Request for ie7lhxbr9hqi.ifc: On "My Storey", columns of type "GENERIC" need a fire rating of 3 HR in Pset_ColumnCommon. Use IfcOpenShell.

First a look at what the model holds.

```python
import ifcopenshell
import ifcopenshell.util.element

model = ifcopenshell.open("ie7lhxbr9hqi.ifc")
print(model.schema)
storey = next(s for s in model.by_type("IfcBuildingStorey") if s.Name == "My Storey")
columns = [e for e in ifcopenshell.util.element.get_decomposition(storey) if e.is_a("IfcColumn")]
seen = {}
for e in columns:
    element_type = ifcopenshell.util.element.get_type(e)
    key = (element_type.Name if element_type != e and element_type else None, ifcopenshell.util.element.get_pset(e, "Pset_ColumnCommon", "FireRating"))
    seen[key] = seen.get(key, 0) + 1
for (name, value), count in sorted(seen.items(), key=str):
    print(count, "x", name, "|", value)
```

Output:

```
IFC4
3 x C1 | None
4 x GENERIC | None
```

```python
import ifcopenshell
import ifcopenshell.api.pset
import ifcopenshell.util.element

model = ifcopenshell.open("ie7lhxbr9hqi.ifc")

storey = next(s for s in model.by_type("IfcBuildingStorey") if s.Name == "My Storey")
columns = [e for e in ifcopenshell.util.element.get_decomposition(storey) if e.is_a("IfcColumn")]

count = 0
for e in columns:
    element_type = ifcopenshell.util.element.get_type(e)
    if element_type in (None, e) or element_type.Name != "GENERIC":
        continue
    # add_pset returns the element's existing set when there is one.
    pset = ifcopenshell.api.pset.add_pset(model, product=e, name="Pset_ColumnCommon")
    ifcopenshell.api.pset.edit_pset(model, pset=pset, properties={"FireRating": "3 HR"})
    count += 1

print(count, "columns updated")

model.write("ie7lhxbr9hqi_edited.ifc")
```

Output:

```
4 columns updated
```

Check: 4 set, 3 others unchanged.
